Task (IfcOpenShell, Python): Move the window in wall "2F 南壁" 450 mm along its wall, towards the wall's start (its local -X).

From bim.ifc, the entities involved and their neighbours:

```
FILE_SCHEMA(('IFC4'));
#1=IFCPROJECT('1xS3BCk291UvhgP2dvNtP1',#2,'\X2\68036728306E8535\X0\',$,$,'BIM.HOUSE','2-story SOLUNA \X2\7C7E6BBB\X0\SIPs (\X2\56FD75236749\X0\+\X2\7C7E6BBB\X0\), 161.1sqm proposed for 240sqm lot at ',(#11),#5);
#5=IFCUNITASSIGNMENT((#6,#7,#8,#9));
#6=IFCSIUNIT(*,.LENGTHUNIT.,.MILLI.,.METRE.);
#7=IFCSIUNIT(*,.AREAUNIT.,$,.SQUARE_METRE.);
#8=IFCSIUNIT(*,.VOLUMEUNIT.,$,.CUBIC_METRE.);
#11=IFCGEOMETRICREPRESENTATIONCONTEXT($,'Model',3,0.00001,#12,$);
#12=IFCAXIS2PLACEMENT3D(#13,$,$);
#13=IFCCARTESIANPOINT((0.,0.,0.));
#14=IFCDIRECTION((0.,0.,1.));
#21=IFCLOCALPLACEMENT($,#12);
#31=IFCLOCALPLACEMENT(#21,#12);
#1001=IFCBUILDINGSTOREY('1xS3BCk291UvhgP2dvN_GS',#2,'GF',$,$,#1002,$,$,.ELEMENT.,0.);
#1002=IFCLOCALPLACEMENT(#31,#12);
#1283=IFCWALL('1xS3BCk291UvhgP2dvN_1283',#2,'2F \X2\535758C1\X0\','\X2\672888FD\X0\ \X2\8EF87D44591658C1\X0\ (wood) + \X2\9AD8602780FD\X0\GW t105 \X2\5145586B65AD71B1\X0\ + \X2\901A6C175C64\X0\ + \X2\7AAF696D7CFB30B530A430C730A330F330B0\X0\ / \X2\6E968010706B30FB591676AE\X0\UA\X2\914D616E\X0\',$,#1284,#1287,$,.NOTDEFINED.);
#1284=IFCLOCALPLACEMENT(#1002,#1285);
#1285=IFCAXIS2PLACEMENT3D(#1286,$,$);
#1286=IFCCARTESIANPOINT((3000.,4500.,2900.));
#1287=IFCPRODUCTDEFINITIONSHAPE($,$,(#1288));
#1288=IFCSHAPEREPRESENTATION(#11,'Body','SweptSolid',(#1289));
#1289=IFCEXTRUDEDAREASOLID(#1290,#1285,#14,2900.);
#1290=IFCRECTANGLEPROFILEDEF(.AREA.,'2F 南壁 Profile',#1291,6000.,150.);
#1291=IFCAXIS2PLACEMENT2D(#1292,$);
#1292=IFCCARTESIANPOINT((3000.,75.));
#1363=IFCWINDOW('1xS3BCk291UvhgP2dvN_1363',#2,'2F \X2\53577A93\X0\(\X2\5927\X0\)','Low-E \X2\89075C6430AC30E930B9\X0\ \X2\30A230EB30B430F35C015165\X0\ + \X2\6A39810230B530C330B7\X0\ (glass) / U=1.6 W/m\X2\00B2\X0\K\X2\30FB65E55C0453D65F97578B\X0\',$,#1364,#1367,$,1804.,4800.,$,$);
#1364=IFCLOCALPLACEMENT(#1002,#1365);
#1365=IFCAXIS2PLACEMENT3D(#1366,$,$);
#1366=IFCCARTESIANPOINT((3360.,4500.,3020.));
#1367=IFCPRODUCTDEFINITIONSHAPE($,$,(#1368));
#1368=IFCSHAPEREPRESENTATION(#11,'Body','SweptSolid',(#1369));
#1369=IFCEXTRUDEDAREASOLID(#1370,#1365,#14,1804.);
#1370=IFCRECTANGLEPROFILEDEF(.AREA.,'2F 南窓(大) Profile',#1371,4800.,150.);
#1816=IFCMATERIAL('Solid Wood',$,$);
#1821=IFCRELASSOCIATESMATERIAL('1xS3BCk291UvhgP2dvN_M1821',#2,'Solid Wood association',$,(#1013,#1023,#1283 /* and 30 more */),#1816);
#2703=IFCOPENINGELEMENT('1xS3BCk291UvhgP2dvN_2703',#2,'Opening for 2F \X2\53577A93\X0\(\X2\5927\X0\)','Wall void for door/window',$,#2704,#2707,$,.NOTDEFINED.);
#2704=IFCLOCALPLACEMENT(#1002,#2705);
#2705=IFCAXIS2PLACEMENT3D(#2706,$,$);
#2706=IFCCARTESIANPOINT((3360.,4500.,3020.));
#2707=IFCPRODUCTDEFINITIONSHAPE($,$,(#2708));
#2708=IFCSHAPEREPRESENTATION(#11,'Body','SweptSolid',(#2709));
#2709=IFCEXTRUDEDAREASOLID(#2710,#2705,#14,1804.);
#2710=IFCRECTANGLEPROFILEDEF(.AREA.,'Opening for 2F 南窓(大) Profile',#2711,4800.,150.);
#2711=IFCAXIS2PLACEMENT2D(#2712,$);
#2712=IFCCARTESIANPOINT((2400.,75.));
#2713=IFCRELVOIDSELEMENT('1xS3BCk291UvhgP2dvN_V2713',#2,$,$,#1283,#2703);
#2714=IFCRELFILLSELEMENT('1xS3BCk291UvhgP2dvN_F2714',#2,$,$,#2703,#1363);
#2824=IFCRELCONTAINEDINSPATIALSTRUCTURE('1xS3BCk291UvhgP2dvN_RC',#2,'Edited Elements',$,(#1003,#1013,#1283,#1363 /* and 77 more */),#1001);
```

```python
import ifcopenshell
import ifcopenshell.api.geometry
import ifcopenshell.util.placement

model = ifcopenshell.open("bim.ifc")

window = model.by_id(1363)
opening = window.FillsVoids[0].RelatingOpeningElement
wall = opening.VoidsElements[0].RelatingBuildingElement

wall_matrix = ifcopenshell.util.placement.get_local_placement(wall.ObjectPlacement)
shift = wall_matrix[:3, 0] * -450.0
before = ifcopenshell.util.placement.get_local_placement(window.ObjectPlacement)[:3, 3].copy()

# The window is not placed relative to its opening, so move both.
for product in (opening, window):
    matrix = ifcopenshell.util.placement.get_local_placement(product.ObjectPlacement)
    matrix[:3, 3] += shift
    ifcopenshell.api.geometry.edit_object_placement(model, product=product, matrix=matrix, is_si=False)

after = ifcopenshell.util.placement.get_local_placement(window.ObjectPlacement)[:3, 3]
print("window moved by", (after - before).round(3) + 0.0)

model.write("bim_v2.ifc")
```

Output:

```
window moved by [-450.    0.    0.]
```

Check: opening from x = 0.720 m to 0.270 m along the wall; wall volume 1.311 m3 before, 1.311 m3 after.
